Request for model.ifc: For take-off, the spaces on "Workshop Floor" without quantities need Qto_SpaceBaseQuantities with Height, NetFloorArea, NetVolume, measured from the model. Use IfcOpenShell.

First a look at what the model holds.

```python
import ifcopenshell
import ifcopenshell.util.element
import ifcopenshell.util.unit

model = ifcopenshell.open("model.ifc")
print(model.schema)
for unit_type in ("LENGTHUNIT", "AREAUNIT", "VOLUMEUNIT"):
    print(unit_type, ifcopenshell.util.unit.calculate_unit_scale(model, unit_type))
storey = next(s for s in model.by_type("IfcBuildingStorey") if s.Name == "Workshop Floor")
spaces = [e for e in ifcopenshell.util.element.get_decomposition(storey) if e.is_a("IfcSpace")]
for e in sorted(spaces, key=lambda e: e.id()):
    print(e.id(), e.is_a(), e.Name, list(ifcopenshell.util.element.get_psets(e, qtos_only=True)), sep=" | ")
```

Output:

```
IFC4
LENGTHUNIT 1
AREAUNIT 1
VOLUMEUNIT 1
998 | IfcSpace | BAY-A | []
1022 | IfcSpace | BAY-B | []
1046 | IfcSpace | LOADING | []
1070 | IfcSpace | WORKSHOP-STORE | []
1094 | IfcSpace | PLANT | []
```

```python
import ifcopenshell
import ifcopenshell.api.pset
import ifcopenshell.geom
import ifcopenshell.util.element
import ifcopenshell.util.shape
import ifcopenshell.util.unit

model = ifcopenshell.open("model.ifc")
unit_scale = ifcopenshell.util.unit.calculate_unit_scale(model)
area_scale = ifcopenshell.util.unit.calculate_unit_scale(model, "AREAUNIT")
volume_scale = ifcopenshell.util.unit.calculate_unit_scale(model, "VOLUMEUNIT")
settings = ifcopenshell.geom.settings()

storey = next(s for s in model.by_type("IfcBuildingStorey") if s.Name == "Workshop Floor")
spaces = [e for e in ifcopenshell.util.element.get_decomposition(storey) if e.is_a("IfcSpace")]

for e in sorted(spaces, key=lambda e: e.id()):
    if ifcopenshell.util.element.get_psets(e, qtos_only=True, should_inherit=False):
        continue
    # Geometry comes back in metres, in the element's own axes.
    shape = ifcopenshell.geom.create_shape(settings, e)
    values = {
        "Height": ifcopenshell.util.shape.get_z(shape.geometry) / unit_scale,
        "NetFloorArea": ifcopenshell.util.shape.get_footprint_area(shape.geometry) / area_scale,
        "NetVolume": ifcopenshell.util.shape.get_volume(shape.geometry) / volume_scale,
    }
    qto = ifcopenshell.api.pset.add_qto(model, product=e, name="Qto_SpaceBaseQuantities")
    ifcopenshell.api.pset.edit_qto(model, qto=qto, properties=values)
    print(e.id(), {k: round(v, 3) for k, v in values.items()})

model.write("model-out.ifc")
```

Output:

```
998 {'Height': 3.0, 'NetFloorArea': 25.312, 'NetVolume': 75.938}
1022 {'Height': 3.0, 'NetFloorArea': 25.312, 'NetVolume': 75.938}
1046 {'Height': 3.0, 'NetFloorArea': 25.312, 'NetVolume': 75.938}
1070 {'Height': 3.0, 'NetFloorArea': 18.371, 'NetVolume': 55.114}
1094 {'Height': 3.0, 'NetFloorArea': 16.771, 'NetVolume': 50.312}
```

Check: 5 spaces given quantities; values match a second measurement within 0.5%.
